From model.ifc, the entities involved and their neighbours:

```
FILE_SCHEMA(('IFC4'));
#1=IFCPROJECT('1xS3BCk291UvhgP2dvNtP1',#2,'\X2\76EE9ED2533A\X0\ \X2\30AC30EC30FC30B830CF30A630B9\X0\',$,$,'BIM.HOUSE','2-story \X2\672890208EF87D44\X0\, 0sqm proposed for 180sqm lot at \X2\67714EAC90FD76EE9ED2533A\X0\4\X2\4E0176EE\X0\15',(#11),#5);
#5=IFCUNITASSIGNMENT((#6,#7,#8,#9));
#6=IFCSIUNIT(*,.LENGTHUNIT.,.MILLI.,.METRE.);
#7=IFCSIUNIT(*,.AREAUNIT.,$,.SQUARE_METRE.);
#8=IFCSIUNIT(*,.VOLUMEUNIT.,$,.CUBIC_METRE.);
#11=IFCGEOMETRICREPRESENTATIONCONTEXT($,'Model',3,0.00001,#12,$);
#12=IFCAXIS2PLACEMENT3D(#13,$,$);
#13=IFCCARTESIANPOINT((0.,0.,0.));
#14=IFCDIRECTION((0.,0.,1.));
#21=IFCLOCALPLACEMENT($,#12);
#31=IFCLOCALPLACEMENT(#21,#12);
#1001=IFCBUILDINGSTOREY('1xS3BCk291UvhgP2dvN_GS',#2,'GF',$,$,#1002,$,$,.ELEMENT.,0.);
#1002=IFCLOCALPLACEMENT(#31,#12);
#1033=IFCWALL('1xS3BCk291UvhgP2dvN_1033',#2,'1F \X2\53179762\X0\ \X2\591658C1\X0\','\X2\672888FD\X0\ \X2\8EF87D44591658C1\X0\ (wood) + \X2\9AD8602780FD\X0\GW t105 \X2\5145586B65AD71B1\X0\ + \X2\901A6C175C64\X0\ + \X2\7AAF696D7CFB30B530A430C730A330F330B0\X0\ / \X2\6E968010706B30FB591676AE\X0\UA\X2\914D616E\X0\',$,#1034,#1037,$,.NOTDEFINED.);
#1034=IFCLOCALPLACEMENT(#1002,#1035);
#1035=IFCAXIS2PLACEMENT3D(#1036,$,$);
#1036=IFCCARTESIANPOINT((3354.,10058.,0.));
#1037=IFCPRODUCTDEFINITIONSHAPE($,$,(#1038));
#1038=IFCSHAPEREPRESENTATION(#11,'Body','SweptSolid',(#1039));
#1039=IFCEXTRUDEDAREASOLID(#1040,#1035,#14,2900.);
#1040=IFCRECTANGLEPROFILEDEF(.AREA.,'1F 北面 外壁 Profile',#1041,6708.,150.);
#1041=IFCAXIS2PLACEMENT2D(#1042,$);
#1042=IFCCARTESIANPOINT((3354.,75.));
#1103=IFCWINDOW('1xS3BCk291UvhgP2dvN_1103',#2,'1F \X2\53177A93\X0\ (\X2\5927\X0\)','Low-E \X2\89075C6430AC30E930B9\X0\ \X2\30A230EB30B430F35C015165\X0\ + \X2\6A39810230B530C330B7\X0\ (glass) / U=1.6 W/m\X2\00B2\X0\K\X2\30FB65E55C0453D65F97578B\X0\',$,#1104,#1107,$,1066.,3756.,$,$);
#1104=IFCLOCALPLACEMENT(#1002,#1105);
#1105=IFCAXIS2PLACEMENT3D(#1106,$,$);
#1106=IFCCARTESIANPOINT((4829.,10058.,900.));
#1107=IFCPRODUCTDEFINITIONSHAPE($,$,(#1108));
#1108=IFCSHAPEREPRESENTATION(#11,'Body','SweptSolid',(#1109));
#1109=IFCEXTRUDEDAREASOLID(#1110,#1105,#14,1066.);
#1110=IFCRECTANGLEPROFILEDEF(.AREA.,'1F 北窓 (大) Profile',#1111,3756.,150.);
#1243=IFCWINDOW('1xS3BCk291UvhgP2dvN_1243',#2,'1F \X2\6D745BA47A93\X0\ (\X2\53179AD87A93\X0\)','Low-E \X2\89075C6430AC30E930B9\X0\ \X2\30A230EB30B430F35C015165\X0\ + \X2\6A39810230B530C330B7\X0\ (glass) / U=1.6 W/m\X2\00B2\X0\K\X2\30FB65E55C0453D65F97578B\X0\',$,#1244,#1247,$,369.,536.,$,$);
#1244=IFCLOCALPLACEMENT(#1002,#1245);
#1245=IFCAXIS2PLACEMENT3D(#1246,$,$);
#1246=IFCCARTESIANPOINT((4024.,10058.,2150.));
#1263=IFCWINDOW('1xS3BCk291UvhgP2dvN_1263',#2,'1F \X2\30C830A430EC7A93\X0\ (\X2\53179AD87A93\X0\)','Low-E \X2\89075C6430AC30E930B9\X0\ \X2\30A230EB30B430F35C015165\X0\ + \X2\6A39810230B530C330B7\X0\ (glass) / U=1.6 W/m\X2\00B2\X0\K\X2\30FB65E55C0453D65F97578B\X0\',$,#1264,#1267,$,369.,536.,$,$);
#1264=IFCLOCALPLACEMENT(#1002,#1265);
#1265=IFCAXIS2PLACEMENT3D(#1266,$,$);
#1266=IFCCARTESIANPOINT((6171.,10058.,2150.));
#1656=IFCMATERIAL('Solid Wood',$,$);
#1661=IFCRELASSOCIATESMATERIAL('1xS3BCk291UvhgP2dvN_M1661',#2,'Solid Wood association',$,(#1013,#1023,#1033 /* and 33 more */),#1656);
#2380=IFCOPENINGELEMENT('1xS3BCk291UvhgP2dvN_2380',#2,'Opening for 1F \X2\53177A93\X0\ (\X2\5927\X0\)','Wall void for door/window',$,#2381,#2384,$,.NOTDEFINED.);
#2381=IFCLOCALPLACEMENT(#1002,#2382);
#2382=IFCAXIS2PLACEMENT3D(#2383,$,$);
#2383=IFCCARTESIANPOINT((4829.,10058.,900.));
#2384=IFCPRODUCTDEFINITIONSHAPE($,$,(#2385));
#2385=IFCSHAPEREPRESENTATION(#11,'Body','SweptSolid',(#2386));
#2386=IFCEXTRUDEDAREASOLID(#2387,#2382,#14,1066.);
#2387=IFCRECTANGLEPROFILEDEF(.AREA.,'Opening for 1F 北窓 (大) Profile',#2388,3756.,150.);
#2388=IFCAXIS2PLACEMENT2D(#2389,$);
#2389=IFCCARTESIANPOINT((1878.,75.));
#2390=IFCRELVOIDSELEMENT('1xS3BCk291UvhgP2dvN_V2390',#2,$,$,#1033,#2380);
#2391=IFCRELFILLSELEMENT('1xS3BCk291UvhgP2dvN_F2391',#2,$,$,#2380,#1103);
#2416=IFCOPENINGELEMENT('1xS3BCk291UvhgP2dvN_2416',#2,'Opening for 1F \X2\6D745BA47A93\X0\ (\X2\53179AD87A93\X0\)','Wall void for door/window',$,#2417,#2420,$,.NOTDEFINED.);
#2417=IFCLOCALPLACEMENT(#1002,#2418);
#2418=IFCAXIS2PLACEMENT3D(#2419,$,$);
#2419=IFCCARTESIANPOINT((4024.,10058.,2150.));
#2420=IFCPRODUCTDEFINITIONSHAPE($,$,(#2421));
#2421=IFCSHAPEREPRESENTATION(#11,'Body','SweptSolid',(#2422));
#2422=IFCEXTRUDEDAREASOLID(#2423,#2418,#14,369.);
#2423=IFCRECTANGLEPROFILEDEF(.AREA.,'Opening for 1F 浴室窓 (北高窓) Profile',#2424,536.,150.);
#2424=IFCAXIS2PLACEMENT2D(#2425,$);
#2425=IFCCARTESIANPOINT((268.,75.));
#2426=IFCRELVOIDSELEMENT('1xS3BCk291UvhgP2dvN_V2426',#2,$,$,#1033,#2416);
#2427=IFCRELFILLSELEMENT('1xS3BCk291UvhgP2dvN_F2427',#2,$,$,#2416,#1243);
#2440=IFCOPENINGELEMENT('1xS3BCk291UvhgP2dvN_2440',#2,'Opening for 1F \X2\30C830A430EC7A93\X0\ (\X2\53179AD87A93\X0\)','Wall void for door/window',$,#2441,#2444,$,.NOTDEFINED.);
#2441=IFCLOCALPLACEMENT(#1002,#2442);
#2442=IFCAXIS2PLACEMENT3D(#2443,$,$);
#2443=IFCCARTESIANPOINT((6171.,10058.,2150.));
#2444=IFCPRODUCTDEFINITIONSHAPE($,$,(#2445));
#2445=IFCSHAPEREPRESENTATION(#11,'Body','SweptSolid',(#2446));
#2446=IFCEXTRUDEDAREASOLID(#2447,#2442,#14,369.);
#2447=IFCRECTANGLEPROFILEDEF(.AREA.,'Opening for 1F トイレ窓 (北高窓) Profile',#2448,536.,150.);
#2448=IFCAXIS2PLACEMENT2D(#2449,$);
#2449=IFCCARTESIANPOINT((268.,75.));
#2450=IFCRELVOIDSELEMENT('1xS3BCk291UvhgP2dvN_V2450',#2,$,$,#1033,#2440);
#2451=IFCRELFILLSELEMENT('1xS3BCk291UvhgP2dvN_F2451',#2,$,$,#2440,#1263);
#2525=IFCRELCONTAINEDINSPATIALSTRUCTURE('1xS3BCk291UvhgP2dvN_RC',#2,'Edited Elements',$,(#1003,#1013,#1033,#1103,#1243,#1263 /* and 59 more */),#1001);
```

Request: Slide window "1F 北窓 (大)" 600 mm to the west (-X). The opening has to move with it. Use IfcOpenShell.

```python
import ifcopenshell
import ifcopenshell.api.geometry
import ifcopenshell.util.placement
import ifcopenshell.util.unit

model = ifcopenshell.open("model.ifc")
unit_scale = ifcopenshell.util.unit.calculate_unit_scale(model)

window = model.by_guid("1xS3BCk291UvhgP2dvN_1103")
opening = window.FillsVoids[0].RelatingOpeningElement
wall = opening.VoidsElements[0].RelatingBuildingElement

wall_matrix = ifcopenshell.util.placement.get_local_placement(wall.ObjectPlacement)
shift = wall_matrix[:3, 0] * -0.6 / unit_scale
before = ifcopenshell.util.placement.get_local_placement(window.ObjectPlacement)[:3, 3].copy()

# The window is not placed relative to its opening, so move both.
for product in (opening, window):
    matrix = ifcopenshell.util.placement.get_local_placement(product.ObjectPlacement)
    matrix[:3, 3] += shift
    ifcopenshell.api.geometry.edit_object_placement(model, product=product, matrix=matrix, is_si=False)

after = ifcopenshell.util.placement.get_local_placement(window.ObjectPlacement)[:3, 3]
print("window moved by", (after - before).round(3) + 0.0)

model.write("model-out.ifc")
```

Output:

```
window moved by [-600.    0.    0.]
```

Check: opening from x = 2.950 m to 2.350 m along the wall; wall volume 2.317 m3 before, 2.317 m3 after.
